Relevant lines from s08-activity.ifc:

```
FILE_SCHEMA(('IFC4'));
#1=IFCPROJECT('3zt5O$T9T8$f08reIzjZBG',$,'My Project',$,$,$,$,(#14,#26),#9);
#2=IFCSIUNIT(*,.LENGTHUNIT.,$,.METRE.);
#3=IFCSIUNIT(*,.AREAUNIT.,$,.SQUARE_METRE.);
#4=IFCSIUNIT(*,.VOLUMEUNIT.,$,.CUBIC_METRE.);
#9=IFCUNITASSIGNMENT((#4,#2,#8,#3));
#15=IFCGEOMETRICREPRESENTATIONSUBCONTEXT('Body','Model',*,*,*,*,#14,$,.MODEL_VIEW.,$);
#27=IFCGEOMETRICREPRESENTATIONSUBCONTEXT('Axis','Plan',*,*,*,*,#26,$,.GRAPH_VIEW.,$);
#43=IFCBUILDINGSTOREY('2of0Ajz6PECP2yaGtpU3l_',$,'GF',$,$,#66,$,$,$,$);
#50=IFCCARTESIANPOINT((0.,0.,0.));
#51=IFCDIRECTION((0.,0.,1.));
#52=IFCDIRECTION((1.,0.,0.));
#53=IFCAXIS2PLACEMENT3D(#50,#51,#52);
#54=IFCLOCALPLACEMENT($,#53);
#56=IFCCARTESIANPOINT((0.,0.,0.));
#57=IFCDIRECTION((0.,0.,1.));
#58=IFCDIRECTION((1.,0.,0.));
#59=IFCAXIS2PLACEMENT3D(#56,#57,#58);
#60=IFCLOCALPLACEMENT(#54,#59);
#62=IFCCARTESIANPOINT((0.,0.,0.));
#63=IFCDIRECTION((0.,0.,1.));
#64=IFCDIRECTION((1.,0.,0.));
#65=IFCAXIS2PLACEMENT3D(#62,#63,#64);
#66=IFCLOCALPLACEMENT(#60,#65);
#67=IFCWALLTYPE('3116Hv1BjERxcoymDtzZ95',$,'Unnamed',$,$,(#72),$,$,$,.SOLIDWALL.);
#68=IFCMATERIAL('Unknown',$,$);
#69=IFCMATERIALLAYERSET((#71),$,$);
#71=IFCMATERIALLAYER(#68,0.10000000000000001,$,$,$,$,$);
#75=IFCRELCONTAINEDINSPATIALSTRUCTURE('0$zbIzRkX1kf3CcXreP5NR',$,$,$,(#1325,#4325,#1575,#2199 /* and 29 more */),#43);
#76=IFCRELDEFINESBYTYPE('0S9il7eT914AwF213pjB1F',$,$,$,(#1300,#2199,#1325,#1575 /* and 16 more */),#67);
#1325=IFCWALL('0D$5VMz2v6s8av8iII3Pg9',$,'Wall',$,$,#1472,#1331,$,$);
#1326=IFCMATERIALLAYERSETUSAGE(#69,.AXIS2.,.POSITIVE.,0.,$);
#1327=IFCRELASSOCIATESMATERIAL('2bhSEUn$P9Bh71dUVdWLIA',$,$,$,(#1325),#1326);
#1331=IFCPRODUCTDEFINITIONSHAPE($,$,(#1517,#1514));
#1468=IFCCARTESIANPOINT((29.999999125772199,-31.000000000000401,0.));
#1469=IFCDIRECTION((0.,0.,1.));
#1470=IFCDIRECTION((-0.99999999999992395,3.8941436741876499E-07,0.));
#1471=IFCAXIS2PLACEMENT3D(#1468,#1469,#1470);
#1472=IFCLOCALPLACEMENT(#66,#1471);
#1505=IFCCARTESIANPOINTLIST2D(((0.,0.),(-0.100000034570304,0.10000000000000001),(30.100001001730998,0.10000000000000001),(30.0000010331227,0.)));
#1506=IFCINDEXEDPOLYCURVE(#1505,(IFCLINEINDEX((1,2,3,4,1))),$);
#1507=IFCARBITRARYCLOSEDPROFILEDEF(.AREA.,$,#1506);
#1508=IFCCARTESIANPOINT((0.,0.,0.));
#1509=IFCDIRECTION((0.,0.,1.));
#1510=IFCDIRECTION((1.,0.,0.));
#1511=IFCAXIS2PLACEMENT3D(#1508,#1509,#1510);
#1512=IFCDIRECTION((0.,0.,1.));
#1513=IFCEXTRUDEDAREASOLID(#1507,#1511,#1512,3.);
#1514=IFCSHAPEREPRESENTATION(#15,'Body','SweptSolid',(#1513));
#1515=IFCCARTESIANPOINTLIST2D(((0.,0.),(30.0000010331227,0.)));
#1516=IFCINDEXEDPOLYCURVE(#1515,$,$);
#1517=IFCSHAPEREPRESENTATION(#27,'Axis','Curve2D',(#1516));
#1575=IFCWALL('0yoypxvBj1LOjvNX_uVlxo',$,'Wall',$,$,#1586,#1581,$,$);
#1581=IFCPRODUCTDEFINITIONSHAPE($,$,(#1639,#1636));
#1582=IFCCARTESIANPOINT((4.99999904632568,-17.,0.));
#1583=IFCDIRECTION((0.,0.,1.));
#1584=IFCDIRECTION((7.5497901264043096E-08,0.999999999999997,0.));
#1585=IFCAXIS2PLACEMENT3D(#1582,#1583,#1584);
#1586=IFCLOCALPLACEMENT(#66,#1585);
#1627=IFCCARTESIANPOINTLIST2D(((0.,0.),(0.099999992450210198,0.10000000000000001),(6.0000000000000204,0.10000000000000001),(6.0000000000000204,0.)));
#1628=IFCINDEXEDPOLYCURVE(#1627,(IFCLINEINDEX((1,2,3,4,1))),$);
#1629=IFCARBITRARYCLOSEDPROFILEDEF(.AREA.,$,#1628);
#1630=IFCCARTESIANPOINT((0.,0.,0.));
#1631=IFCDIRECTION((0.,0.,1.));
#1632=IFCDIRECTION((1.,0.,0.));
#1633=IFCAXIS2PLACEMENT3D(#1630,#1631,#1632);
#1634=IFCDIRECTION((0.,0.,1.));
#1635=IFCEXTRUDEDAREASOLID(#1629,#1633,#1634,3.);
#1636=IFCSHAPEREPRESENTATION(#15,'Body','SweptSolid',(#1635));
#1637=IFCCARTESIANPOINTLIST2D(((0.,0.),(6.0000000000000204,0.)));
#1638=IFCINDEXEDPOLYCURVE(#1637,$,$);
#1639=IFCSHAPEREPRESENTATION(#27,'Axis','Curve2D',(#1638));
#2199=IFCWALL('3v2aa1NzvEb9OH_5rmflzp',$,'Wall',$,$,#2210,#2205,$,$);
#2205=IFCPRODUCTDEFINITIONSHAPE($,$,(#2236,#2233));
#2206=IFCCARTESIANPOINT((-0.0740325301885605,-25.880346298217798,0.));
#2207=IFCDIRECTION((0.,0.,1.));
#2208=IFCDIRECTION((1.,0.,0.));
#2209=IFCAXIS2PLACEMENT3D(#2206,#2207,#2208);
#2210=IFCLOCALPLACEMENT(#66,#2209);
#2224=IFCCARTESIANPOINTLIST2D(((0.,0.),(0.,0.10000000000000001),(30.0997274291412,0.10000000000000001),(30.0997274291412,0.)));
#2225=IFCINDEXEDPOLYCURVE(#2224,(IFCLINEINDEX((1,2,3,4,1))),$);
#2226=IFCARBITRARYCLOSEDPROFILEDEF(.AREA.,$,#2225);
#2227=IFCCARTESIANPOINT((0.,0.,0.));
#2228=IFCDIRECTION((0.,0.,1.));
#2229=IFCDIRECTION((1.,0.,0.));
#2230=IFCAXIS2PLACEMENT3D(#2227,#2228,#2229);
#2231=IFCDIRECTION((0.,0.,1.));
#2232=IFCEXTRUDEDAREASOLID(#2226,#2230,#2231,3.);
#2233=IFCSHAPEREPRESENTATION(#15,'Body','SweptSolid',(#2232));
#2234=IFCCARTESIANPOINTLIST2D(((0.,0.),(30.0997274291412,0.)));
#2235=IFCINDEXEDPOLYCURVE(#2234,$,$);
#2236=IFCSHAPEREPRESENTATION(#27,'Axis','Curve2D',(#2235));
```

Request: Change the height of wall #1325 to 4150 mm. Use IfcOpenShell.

```python
import ifcopenshell
import ifcopenshell.geom
import ifcopenshell.util.representation
import ifcopenshell.util.shape
import ifcopenshell.util.unit

model = ifcopenshell.open("s08-activity.ifc")
unit_scale = ifcopenshell.util.unit.calculate_unit_scale(model)
settings = ifcopenshell.geom.settings()


def volume(element):
    """Net volume in cubic metres, openings subtracted."""
    shape = ifcopenshell.geom.create_shape(settings, element)
    return ifcopenshell.util.shape.get_volume(shape.geometry)


wall = model.by_guid("0D$5VMz2v6s8av8iII3Pg9")
before = volume(wall)

body = ifcopenshell.util.representation.get_representation(wall, "Model", "Body")
solid = body.Items[0]
old_height = solid.Depth
solid.Depth = 4.15 / unit_scale
after = volume(wall)

print(f"height {old_height:g} -> {solid.Depth:g}, volume {before:.3f} -> {after:.3f} m3")

model.write("s08-activity_updated.ifc")
```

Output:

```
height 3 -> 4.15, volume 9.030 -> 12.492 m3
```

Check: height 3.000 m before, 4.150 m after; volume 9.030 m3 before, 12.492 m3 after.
